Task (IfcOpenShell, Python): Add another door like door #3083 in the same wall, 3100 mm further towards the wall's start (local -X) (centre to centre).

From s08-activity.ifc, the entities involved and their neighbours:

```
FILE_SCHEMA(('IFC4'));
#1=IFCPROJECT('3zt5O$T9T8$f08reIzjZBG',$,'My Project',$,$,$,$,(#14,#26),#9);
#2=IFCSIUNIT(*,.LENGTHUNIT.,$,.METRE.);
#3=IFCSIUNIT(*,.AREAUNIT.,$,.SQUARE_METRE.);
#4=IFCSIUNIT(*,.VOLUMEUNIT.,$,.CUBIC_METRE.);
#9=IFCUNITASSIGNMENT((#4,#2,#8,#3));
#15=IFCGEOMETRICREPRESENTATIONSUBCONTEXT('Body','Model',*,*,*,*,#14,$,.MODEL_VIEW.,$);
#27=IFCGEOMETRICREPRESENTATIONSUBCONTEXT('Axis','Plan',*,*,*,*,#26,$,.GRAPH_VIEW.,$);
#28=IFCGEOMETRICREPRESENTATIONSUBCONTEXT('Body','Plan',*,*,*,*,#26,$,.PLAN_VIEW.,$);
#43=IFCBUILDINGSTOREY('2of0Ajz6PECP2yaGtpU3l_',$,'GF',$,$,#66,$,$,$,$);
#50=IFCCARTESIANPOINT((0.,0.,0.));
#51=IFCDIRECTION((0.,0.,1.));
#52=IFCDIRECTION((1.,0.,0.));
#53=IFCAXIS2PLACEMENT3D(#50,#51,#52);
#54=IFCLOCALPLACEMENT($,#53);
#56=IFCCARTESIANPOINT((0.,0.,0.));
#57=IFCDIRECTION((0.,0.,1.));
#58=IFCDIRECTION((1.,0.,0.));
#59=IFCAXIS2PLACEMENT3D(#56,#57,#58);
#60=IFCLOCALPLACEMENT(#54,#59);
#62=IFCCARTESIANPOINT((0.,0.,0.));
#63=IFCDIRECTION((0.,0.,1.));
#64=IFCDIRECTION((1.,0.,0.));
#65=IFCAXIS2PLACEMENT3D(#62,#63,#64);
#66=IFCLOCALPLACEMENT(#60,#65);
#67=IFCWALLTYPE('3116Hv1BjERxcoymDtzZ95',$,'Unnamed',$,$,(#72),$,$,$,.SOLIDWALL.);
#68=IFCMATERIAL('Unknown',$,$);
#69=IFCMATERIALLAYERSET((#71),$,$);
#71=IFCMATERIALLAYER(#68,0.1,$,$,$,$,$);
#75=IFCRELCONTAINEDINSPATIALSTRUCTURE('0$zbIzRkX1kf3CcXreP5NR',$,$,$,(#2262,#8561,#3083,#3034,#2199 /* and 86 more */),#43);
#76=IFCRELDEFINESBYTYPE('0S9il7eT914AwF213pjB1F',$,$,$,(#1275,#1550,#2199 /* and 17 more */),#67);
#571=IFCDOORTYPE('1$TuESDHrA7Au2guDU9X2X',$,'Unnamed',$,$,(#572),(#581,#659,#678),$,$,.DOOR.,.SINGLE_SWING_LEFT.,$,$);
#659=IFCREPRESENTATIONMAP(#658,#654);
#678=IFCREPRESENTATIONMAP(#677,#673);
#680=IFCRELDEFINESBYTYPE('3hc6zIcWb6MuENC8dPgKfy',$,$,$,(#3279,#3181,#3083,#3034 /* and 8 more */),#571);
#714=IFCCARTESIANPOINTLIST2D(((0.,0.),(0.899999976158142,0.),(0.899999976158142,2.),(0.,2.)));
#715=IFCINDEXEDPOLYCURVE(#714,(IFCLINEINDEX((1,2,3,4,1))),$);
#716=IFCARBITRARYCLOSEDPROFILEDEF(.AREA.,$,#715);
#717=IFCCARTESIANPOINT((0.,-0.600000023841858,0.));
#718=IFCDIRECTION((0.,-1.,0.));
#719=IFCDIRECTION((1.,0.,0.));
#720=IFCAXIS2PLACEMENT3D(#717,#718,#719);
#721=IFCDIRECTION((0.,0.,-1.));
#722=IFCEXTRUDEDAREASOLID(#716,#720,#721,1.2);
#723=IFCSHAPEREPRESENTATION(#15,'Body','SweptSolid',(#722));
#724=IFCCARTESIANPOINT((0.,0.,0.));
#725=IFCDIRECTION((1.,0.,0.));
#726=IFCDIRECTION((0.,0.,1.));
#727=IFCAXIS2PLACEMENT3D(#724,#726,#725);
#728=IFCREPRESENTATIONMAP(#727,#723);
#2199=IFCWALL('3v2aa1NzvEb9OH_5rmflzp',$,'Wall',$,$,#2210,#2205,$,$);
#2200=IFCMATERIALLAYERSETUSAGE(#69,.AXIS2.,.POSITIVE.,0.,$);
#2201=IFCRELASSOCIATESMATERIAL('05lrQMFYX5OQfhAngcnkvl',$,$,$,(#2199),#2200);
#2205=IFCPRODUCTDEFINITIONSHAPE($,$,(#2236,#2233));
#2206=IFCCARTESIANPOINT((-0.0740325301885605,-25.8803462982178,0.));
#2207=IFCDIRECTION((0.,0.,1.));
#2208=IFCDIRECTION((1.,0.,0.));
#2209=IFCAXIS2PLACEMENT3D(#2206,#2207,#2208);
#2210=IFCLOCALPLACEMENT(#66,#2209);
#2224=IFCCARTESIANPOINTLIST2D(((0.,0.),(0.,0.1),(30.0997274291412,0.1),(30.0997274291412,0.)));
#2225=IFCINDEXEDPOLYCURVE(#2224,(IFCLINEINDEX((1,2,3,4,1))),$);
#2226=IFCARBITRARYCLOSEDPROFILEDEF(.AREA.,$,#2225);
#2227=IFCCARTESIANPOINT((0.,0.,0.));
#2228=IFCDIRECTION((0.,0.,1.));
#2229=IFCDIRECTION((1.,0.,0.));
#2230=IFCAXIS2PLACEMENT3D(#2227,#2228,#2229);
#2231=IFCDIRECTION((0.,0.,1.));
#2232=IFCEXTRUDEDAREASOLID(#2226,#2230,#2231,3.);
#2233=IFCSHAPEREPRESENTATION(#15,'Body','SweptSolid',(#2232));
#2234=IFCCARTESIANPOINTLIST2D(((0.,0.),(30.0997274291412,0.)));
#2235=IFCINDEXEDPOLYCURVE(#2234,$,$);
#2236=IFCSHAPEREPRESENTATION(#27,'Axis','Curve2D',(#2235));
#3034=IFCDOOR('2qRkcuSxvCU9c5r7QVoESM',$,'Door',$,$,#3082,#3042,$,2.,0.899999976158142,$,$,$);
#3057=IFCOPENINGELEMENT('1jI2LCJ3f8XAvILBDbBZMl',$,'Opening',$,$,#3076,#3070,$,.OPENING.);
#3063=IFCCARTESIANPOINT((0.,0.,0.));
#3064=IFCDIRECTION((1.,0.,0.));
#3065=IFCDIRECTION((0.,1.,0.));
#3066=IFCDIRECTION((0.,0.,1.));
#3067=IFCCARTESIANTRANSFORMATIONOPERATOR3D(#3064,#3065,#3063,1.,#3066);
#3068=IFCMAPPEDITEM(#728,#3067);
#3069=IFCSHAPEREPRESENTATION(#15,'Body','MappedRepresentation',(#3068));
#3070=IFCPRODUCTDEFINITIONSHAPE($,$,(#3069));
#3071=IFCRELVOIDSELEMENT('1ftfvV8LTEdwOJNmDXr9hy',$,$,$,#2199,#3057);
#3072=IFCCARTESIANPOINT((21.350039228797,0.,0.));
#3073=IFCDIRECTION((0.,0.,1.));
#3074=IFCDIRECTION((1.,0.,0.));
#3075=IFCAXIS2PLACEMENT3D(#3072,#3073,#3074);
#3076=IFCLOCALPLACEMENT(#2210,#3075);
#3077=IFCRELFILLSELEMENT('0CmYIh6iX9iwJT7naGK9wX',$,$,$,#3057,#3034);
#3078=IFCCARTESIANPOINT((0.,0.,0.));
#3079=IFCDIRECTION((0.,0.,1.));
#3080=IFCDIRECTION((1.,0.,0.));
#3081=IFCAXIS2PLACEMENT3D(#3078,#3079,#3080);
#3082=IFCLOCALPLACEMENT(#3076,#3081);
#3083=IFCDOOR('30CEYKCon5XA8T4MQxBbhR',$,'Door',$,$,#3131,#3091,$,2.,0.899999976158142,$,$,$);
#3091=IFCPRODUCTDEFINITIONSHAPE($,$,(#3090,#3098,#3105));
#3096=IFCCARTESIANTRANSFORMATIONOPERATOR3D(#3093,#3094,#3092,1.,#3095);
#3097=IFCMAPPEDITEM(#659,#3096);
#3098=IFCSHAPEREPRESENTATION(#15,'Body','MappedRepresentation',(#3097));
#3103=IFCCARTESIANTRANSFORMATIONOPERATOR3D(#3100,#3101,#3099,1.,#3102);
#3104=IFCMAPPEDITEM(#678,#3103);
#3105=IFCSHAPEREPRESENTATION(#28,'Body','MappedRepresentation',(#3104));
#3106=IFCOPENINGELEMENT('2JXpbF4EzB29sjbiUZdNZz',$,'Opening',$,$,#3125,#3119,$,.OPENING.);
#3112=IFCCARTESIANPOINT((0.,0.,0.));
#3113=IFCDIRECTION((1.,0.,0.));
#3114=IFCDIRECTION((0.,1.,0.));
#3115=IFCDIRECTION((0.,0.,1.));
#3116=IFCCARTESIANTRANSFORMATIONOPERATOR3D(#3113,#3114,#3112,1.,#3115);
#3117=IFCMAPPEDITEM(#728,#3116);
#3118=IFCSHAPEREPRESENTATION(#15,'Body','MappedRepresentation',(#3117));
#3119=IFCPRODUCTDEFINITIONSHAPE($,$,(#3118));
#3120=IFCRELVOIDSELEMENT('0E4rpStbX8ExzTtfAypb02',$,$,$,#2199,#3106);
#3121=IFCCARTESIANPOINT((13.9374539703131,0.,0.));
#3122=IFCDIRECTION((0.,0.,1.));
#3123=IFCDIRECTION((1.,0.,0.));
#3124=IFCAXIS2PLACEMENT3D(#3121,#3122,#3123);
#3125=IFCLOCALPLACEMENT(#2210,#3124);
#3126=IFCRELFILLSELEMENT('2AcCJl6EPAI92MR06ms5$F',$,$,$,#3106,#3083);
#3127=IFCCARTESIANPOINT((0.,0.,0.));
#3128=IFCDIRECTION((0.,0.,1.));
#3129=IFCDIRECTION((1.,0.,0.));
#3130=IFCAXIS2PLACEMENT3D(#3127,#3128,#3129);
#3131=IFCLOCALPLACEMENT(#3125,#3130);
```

```python
import ifcopenshell
import ifcopenshell.api.feature
import ifcopenshell.api.geometry
import ifcopenshell.api.root
import ifcopenshell.geom
import ifcopenshell.util.element
import ifcopenshell.util.placement
import ifcopenshell.util.shape
import ifcopenshell.util.unit

model = ifcopenshell.open("s08-activity.ifc")
unit_scale = ifcopenshell.util.unit.calculate_unit_scale(model)
settings = ifcopenshell.geom.settings()


def volume(element):
    """Net volume in cubic metres, openings subtracted."""
    shape = ifcopenshell.geom.create_shape(settings, element)
    return ifcopenshell.util.shape.get_volume(shape.geometry)


door = model.by_guid("30CEYKCon5XA8T4MQxBbhR")
opening = door.FillsVoids[0].RelatingOpeningElement
wall = opening.VoidsElements[0].RelatingBuildingElement
before = volume(wall)
shift = ifcopenshell.util.placement.get_local_placement(wall.ObjectPlacement)[:3, 0] * -3.1 / unit_scale

# copy_class copies the void relationship, type, container and properties, but no geometry.
new_opening = ifcopenshell.api.root.copy_class(model, product=opening)
new_opening.Representation = ifcopenshell.util.element.copy_deep(
    model, opening.Representation, exclude=["IfcGeometricRepresentationContext", "IfcRepresentationMap"]
)
new_door = ifcopenshell.api.root.copy_class(model, product=door)
new_door.Representation = ifcopenshell.util.element.copy_deep(
    model, door.Representation, exclude=["IfcGeometricRepresentationContext", "IfcRepresentationMap"]
)
ifcopenshell.api.feature.add_filling(model, opening=new_opening, element=new_door)

for old, new in ((opening, new_opening), (door, new_door)):
    matrix = ifcopenshell.util.placement.get_local_placement(old.ObjectPlacement)
    matrix[:3, 3] += shift
    ifcopenshell.api.geometry.edit_object_placement(model, product=new, matrix=matrix, is_si=False)

after = volume(wall)

print(f"wall volume {before:.3f} -> {after:.3f} m3")

model.write("s08-activity_updated.ifc")
```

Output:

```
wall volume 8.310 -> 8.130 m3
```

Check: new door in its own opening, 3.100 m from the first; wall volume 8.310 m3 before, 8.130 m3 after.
